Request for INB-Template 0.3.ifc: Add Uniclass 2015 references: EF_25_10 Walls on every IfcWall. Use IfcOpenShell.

First a look at what the model holds.

```python
import ifcopenshell

model = ifcopenshell.open("INB-Template 0.3.ifc")
print(model.schema)
print("classifications:", [c.Name for c in model.by_type("IfcClassification")])
for ifc_class in ("IfcDoor", "IfcRoof", "IfcStair", "IfcWall", "IfcWindow"):
    print(ifc_class, len(model.by_type(ifc_class)))
```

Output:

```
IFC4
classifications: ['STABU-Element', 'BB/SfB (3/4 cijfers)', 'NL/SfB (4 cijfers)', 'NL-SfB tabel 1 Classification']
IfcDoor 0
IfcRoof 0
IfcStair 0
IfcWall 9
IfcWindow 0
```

```python
import ifcopenshell
import ifcopenshell.api.classification

model = ifcopenshell.open("INB-Template 0.3.ifc")

system = ifcopenshell.api.classification.add_classification(model, classification="Uniclass 2015")

codes = {
    "IfcWall": ("EF_25_10", "Walls"),
}
for ifc_class, (code, name) in codes.items():
    products = model.by_type(ifc_class)
    ifcopenshell.api.classification.add_reference(
        model, products=products, classification=system, identification=code, name=name
    )
    print(code, len(products))

model.write("INB-Template 0.3-out.ifc")
```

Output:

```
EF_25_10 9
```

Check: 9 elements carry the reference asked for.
